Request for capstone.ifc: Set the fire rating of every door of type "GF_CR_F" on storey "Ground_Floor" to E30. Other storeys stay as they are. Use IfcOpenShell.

First a look at what the model holds.

```python
import ifcopenshell
import ifcopenshell.util.element

model = ifcopenshell.open("capstone.ifc")
print(model.schema)
storey = next(s for s in model.by_type("IfcBuildingStorey") if s.Name == "Ground_Floor")
doors = [e for e in ifcopenshell.util.element.get_decomposition(storey) if e.is_a("IfcDoor")]
seen = {}
for e in doors:
    element_type = ifcopenshell.util.element.get_type(e)
    key = (element_type.Name if element_type != e and element_type else None, ifcopenshell.util.element.get_pset(e, "Pset_DoorCommon", "FireRating"))
    seen[key] = seen.get(key, 0) + 1
for (name, value), count in sorted(seen.items(), key=str):
    print(count, "x", name, "|", value)
```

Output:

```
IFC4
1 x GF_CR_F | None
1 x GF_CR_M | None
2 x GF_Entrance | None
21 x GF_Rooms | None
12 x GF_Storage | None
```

```python
import ifcopenshell
import ifcopenshell.api.pset
import ifcopenshell.util.element

model = ifcopenshell.open("capstone.ifc")

storey = next(s for s in model.by_type("IfcBuildingStorey") if s.Name == "Ground_Floor")
doors = [e for e in ifcopenshell.util.element.get_decomposition(storey) if e.is_a("IfcDoor")]

count = 0
for e in doors:
    element_type = ifcopenshell.util.element.get_type(e)
    if element_type in (None, e) or element_type.Name != "GF_CR_F":
        continue
    # add_pset returns the element's existing set when there is one.
    pset = ifcopenshell.api.pset.add_pset(model, product=e, name="Pset_DoorCommon")
    ifcopenshell.api.pset.edit_pset(model, pset=pset, properties={"FireRating": "E30"})
    count += 1

print(count, "doors updated")

model.write("capstone_rev.ifc")
```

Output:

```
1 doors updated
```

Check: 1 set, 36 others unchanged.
